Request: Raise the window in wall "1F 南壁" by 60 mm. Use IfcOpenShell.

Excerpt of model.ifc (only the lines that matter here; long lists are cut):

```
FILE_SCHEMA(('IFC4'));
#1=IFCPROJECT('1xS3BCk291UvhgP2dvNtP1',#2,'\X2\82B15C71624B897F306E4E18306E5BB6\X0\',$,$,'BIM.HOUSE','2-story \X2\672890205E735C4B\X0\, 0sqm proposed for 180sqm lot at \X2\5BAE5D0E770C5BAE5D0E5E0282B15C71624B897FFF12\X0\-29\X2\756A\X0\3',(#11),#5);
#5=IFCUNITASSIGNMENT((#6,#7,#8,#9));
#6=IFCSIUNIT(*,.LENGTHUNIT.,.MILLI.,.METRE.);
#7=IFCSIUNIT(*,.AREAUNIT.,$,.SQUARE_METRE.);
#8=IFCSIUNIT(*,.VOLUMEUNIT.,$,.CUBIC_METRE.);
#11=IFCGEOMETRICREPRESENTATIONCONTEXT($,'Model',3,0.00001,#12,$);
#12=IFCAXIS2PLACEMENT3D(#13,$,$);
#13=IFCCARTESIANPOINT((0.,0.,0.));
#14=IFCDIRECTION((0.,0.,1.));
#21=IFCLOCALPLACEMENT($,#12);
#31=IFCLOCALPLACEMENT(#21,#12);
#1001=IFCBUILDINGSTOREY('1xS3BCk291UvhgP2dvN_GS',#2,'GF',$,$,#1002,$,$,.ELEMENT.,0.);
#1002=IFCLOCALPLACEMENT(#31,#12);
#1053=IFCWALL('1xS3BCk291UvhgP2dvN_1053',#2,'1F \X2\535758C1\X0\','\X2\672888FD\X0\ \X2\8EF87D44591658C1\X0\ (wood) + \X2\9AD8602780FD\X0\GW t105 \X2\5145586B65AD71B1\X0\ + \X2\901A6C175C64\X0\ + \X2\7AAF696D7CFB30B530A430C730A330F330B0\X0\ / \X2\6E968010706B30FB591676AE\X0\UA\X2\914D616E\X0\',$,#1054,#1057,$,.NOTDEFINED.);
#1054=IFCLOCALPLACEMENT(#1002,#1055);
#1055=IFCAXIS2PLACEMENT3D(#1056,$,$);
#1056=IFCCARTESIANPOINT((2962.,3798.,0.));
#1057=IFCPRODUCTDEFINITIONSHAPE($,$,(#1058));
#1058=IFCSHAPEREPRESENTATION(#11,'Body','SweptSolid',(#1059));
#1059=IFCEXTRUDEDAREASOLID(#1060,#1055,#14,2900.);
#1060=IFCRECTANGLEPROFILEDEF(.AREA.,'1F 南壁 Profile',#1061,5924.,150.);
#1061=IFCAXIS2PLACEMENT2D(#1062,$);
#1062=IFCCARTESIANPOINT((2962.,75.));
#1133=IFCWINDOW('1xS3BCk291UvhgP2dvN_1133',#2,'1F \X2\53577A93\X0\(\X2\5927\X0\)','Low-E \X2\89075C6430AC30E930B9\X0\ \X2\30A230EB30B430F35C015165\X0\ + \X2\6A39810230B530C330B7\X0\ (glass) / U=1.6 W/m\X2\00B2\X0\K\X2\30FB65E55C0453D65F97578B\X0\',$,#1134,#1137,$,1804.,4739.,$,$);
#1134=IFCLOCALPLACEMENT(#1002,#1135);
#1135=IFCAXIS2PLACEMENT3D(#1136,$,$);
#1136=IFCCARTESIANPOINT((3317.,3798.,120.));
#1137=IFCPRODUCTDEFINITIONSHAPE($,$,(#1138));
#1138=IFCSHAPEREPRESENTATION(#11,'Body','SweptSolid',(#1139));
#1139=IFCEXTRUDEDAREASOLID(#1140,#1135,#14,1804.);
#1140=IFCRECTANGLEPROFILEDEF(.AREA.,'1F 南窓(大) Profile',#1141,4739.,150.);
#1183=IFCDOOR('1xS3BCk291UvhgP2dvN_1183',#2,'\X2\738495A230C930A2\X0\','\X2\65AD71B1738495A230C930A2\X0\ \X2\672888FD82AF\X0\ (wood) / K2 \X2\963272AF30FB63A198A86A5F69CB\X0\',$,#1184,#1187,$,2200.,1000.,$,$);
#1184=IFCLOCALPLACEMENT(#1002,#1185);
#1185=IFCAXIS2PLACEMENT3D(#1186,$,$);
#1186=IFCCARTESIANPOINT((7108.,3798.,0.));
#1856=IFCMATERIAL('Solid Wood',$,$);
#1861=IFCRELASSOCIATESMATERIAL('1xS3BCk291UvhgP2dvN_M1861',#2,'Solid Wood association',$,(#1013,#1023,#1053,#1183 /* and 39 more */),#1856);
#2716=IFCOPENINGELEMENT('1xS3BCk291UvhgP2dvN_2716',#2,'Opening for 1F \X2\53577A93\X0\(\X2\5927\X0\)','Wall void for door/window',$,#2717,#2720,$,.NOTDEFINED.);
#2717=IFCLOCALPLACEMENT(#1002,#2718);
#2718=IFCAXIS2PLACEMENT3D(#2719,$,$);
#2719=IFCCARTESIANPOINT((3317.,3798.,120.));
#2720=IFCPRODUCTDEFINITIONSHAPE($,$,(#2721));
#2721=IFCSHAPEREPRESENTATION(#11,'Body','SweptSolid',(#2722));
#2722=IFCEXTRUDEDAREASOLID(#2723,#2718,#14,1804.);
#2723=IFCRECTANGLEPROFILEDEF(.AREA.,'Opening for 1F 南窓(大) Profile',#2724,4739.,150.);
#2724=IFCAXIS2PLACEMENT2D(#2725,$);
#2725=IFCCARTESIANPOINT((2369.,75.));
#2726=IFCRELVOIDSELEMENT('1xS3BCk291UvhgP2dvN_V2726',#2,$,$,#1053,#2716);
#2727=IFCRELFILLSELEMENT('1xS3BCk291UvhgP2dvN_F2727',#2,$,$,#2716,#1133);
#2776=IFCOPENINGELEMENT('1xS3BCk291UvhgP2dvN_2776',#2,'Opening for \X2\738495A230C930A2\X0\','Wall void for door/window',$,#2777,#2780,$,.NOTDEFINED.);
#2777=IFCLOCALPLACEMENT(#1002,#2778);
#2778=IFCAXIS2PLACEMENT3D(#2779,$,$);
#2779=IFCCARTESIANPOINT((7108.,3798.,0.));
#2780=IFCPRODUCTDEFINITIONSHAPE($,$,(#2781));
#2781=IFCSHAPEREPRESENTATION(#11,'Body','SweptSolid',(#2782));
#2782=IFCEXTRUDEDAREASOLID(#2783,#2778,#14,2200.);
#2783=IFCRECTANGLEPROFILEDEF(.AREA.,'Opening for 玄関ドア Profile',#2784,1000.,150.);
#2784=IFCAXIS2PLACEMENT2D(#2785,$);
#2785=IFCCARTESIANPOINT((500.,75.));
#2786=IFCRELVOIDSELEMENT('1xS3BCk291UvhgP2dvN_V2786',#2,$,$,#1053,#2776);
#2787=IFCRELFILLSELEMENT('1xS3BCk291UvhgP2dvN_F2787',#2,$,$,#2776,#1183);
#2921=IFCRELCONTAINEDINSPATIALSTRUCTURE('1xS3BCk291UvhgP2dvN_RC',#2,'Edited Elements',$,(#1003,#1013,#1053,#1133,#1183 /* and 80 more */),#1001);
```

```python
import numpy as np
import ifcopenshell
import ifcopenshell.api.geometry
import ifcopenshell.util.placement
import ifcopenshell.util.unit

model = ifcopenshell.open("model.ifc")
unit_scale = ifcopenshell.util.unit.calculate_unit_scale(model)

window = model.by_guid("1xS3BCk291UvhgP2dvN_1133")
opening = window.FillsVoids[0].RelatingOpeningElement
dz = 60.0

shift = np.array([0.0, 0.0, dz])
# The window is not placed relative to its opening, so move both.
for product in (opening, window):
    matrix = ifcopenshell.util.placement.get_local_placement(product.ObjectPlacement)
    matrix[:3, 3] += shift
    ifcopenshell.api.geometry.edit_object_placement(model, product=product, matrix=matrix, is_si=False)

print(f"moved by {dz * unit_scale:+.3f} m")

model.write("model-out.ifc")
```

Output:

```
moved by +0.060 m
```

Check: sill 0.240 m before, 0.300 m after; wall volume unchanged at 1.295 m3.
